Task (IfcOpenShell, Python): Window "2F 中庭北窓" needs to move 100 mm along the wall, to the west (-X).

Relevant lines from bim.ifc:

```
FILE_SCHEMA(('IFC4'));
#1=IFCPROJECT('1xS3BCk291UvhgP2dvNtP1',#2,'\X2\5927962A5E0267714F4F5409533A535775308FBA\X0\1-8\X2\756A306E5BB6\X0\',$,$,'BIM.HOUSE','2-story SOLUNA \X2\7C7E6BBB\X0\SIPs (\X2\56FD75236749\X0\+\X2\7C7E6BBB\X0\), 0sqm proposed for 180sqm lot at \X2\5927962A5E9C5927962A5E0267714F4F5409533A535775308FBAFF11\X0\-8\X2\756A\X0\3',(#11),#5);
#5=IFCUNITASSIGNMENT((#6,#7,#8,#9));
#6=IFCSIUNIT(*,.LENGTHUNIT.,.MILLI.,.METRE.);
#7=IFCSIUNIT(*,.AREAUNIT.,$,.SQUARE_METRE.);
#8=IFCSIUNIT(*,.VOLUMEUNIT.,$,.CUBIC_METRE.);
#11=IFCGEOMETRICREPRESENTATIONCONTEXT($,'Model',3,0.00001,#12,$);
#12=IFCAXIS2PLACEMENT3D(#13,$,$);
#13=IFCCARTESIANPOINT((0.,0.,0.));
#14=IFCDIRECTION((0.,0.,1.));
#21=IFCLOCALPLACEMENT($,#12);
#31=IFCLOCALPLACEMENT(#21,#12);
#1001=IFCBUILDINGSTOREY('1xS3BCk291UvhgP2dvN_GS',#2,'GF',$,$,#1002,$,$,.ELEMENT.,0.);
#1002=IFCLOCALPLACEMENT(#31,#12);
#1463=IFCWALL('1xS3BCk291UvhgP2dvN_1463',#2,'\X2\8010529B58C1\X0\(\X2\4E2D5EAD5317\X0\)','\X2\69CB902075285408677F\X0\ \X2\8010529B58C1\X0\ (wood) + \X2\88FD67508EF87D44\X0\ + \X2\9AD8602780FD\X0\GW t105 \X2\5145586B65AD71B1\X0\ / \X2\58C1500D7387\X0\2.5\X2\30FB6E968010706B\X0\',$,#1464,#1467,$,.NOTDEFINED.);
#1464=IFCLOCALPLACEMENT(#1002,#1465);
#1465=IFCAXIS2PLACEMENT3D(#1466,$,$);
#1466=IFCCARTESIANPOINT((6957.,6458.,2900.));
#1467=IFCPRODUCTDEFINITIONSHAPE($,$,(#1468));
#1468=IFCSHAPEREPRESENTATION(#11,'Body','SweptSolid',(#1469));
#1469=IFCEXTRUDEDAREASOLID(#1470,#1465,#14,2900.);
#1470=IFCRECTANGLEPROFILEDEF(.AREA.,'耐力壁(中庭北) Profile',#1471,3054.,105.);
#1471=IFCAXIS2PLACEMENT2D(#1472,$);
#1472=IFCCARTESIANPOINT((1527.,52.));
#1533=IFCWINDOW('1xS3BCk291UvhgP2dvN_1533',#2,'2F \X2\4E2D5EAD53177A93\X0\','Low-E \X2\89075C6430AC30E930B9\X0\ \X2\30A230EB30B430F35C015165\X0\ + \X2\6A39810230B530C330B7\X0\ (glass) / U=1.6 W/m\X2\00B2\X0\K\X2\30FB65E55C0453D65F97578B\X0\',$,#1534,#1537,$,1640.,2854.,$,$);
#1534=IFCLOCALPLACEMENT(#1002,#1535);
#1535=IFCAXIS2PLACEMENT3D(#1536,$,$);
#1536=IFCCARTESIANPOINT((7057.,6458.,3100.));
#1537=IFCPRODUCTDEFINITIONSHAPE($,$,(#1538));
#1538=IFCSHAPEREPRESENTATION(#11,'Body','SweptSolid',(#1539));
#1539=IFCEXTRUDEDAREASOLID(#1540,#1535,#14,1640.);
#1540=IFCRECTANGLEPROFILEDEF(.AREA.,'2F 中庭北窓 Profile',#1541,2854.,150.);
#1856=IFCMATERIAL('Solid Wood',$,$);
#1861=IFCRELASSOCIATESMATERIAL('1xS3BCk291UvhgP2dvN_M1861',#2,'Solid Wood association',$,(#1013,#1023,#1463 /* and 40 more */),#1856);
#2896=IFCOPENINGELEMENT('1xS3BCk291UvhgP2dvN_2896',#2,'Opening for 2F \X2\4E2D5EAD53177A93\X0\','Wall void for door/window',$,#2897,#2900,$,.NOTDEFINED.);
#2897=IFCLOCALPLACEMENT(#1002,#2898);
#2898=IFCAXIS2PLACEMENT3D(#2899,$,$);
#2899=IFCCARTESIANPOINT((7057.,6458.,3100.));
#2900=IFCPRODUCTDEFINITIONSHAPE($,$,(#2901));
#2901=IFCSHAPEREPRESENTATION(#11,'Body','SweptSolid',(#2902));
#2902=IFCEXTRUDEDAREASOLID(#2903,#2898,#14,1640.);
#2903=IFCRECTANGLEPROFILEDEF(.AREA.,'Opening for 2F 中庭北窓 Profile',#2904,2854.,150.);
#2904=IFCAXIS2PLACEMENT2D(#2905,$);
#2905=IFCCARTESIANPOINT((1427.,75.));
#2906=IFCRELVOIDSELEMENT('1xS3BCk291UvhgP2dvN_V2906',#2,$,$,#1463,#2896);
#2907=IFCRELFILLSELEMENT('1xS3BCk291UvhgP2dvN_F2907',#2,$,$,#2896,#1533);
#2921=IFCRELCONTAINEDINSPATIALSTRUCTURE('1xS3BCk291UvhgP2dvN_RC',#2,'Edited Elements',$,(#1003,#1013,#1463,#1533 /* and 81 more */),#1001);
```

```python
import ifcopenshell
import ifcopenshell.api.geometry
import ifcopenshell.util.placement
import ifcopenshell.util.unit

model = ifcopenshell.open("bim.ifc")
unit_scale = ifcopenshell.util.unit.calculate_unit_scale(model)

window = model.by_guid("1xS3BCk291UvhgP2dvN_1533")
opening = window.FillsVoids[0].RelatingOpeningElement
wall = opening.VoidsElements[0].RelatingBuildingElement

wall_matrix = ifcopenshell.util.placement.get_local_placement(wall.ObjectPlacement)
shift = wall_matrix[:3, 0] * -0.1 / unit_scale
before = ifcopenshell.util.placement.get_local_placement(window.ObjectPlacement)[:3, 3].copy()

# The window is not placed relative to its opening, so move both.
for product in (opening, window):
    matrix = ifcopenshell.util.placement.get_local_placement(product.ObjectPlacement)
    matrix[:3, 3] += shift
    ifcopenshell.api.geometry.edit_object_placement(model, product=product, matrix=matrix, is_si=False)

after = ifcopenshell.util.placement.get_local_placement(window.ObjectPlacement)[:3, 3]
print("window moved by", (after - before).round(3) + 0.0)

model.write("bim_updated.ifc")
```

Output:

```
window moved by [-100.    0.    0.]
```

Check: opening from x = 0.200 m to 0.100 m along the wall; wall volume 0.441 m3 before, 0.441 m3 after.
